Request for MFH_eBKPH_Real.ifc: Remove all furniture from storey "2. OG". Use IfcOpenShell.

First a look at what the model holds.

```python
import ifcopenshell
import ifcopenshell.util.element

model = ifcopenshell.open("MFH_eBKPH_Real.ifc")
print(model.schema)
storey = next(s for s in model.by_type("IfcBuildingStorey") if s.Name == "2. OG")
furniture = [e for e in ifcopenshell.util.element.get_decomposition(storey) if e.is_a("IfcFurnishingElement")]
seen = {}
for e in furniture:
    element_type = ifcopenshell.util.element.get_type(e)
    name = element_type.Name if element_type not in (None, e) else None
    seen[name] = seen.get(name, 0) + 1
for name, count in sorted(seen.items(), key=str):
    print(count, "x", name)
```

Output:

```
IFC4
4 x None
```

```python
import ifcopenshell
import ifcopenshell.api.root
import ifcopenshell.util.element

model = ifcopenshell.open("MFH_eBKPH_Real.ifc")

storey = next(s for s in model.by_type("IfcBuildingStorey") if s.Name == "2. OG")
furniture = [e for e in ifcopenshell.util.element.get_decomposition(storey) if e.is_a("IfcFurnishingElement")]

for e in furniture:
    ifcopenshell.api.root.remove_product(model, product=e)
print(len(furniture), "removed")

model.write("MFH_eBKPH_Real_edited.ifc")
```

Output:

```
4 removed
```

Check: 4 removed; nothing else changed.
